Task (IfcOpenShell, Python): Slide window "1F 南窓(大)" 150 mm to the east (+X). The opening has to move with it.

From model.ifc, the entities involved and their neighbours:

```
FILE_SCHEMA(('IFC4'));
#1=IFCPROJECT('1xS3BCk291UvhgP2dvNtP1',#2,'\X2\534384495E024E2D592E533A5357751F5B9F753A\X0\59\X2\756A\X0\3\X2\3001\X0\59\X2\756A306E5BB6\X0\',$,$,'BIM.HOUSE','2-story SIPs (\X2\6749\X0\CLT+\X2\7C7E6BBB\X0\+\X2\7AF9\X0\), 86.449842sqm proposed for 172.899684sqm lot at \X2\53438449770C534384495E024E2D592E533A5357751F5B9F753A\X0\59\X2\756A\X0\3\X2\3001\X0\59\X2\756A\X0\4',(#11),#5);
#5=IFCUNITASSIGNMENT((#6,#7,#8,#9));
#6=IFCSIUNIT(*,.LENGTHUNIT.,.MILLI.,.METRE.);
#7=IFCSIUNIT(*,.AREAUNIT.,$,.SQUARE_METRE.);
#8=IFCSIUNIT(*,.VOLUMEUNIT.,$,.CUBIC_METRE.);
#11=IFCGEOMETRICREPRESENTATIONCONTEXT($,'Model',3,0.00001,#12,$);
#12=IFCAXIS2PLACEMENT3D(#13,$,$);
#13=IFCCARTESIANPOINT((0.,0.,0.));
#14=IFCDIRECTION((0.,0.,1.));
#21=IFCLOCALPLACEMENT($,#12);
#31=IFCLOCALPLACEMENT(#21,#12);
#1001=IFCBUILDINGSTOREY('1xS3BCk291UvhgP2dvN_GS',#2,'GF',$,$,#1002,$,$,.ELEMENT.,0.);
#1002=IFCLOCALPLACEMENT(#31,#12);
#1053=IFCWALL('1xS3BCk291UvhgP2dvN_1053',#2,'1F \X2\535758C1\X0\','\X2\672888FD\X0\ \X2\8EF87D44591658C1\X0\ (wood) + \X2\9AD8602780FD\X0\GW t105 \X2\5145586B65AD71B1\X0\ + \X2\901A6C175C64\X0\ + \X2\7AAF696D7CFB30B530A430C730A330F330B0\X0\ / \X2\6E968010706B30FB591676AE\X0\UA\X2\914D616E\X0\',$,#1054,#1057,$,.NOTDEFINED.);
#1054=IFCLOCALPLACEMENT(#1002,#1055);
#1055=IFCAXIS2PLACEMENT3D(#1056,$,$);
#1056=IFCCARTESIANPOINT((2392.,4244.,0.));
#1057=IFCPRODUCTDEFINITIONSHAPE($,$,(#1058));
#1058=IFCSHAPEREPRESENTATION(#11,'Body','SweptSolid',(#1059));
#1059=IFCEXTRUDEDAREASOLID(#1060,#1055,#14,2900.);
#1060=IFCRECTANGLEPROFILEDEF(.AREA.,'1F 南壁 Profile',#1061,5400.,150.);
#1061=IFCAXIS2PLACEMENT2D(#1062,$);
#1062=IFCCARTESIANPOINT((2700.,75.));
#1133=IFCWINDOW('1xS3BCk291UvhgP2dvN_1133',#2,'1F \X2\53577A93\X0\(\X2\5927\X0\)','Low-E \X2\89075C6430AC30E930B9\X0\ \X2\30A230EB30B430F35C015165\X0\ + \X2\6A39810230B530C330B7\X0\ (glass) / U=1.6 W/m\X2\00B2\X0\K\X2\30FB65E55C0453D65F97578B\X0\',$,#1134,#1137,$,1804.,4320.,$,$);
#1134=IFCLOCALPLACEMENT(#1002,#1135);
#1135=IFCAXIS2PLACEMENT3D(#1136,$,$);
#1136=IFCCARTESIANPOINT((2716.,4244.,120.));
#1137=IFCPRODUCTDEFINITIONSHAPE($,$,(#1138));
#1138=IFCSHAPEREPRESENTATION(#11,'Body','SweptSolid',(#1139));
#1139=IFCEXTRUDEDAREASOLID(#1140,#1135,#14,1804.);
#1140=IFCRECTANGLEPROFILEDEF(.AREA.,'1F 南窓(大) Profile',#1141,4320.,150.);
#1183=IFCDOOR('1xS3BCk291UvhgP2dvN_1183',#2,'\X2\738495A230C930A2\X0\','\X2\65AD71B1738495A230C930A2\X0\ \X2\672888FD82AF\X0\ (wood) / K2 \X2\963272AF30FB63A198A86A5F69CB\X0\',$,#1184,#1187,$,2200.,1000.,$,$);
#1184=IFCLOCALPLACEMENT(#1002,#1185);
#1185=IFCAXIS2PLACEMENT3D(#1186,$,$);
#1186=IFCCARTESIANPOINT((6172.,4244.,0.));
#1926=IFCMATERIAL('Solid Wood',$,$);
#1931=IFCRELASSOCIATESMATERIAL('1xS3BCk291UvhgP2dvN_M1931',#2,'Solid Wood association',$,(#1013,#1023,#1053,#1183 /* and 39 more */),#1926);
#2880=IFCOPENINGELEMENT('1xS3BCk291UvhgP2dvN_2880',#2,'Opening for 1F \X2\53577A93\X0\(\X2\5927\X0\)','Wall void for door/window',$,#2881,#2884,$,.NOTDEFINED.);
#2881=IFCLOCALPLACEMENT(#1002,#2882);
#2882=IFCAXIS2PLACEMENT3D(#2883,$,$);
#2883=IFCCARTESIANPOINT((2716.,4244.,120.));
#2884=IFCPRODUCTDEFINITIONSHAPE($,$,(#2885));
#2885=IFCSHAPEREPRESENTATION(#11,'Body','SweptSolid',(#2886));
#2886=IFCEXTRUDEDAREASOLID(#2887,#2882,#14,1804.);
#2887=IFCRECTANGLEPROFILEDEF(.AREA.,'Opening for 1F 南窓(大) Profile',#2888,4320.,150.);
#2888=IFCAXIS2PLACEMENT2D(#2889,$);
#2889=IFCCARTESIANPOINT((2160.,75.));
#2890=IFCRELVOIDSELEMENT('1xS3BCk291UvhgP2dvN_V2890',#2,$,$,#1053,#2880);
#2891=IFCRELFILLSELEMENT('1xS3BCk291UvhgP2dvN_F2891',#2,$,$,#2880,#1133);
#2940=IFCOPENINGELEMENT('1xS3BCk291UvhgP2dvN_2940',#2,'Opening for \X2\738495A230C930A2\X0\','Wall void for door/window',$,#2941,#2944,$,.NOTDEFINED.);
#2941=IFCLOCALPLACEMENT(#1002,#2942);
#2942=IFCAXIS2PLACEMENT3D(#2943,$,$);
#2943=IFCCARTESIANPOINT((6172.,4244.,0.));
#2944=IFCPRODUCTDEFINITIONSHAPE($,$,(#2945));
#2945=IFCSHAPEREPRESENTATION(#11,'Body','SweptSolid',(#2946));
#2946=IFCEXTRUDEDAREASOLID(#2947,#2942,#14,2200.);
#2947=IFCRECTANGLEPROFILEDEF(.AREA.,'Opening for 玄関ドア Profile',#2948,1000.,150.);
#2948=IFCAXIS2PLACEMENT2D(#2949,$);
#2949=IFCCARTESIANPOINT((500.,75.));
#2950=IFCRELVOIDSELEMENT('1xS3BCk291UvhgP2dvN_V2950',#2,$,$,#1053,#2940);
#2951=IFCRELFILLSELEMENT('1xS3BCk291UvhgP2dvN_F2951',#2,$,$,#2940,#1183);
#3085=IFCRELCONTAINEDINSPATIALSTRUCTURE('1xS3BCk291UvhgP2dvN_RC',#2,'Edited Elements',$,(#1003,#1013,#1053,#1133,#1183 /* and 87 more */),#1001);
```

```python
import ifcopenshell
import ifcopenshell.api.geometry
import ifcopenshell.util.placement
import ifcopenshell.util.unit

model = ifcopenshell.open("model.ifc")
unit_scale = ifcopenshell.util.unit.calculate_unit_scale(model)

window = model.by_guid("1xS3BCk291UvhgP2dvN_1133")
opening = window.FillsVoids[0].RelatingOpeningElement
wall = opening.VoidsElements[0].RelatingBuildingElement

wall_matrix = ifcopenshell.util.placement.get_local_placement(wall.ObjectPlacement)
shift = wall_matrix[:3, 0] * 0.15 / unit_scale
before = ifcopenshell.util.placement.get_local_placement(window.ObjectPlacement)[:3, 3].copy()

# The window is not placed relative to its opening, so move both.
for product in (opening, window):
    matrix = ifcopenshell.util.placement.get_local_placement(product.ObjectPlacement)
    matrix[:3, 3] += shift
    ifcopenshell.api.geometry.edit_object_placement(model, product=product, matrix=matrix, is_si=False)

after = ifcopenshell.util.placement.get_local_placement(window.ObjectPlacement)[:3, 3]
print("window moved by", (after - before).round(3) + 0.0)

model.write("model_updated.ifc")
```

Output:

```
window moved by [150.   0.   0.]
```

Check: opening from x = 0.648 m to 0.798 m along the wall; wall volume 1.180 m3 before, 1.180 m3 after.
